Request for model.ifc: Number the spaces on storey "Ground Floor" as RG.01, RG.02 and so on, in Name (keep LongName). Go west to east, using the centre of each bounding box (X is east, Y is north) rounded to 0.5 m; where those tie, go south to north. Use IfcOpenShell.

First a look at what the model holds.

```python
import ifcopenshell
import ifcopenshell.util.element
import ifcopenshell.util.placement

model = ifcopenshell.open("model.ifc")
print(model.schema)
storey = next(s for s in model.by_type("IfcBuildingStorey") if s.Name == "Ground Floor")
spaces = [e for e in ifcopenshell.util.element.get_decomposition(storey) if e.is_a("IfcSpace")]
for e in sorted(spaces, key=lambda e: e.id()):
    origin = ifcopenshell.util.placement.get_local_placement(e.ObjectPlacement)[:3, 3]
    print(e.id(), e.Name, e.LongName, origin.round(2) + 0.0, sep=" | ")
```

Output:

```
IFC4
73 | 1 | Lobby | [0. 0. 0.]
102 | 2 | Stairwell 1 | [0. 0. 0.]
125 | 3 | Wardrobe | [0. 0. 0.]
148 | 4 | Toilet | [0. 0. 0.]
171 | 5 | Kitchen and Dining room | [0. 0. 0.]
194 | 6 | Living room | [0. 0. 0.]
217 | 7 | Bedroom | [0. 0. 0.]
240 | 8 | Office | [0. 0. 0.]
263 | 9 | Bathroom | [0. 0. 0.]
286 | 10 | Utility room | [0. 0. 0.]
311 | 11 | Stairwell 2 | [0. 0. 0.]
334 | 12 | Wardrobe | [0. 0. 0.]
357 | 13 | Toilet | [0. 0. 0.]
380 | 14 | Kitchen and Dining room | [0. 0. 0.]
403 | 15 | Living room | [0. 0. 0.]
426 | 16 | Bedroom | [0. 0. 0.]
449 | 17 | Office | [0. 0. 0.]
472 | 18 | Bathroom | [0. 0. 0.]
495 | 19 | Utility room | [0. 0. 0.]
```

```python
import ifcopenshell
import ifcopenshell.geom
import ifcopenshell.util.element
import ifcopenshell.util.shape

model = ifcopenshell.open("model.ifc")
settings = ifcopenshell.geom.settings()
settings.set("use-world-coords", True)


def centre(element):
    shape = ifcopenshell.geom.create_shape(settings, element)
    return ifcopenshell.util.shape.get_bbox_centroid(shape.geometry)


storey = next(s for s in model.by_type("IfcBuildingStorey") if s.Name == "Ground Floor")
spaces = [e for e in ifcopenshell.util.element.get_decomposition(storey) if e.is_a("IfcSpace")]

# Insertion points can sit at a corner or the storey origin, so sort by the geometry (in metres).
centres = {e: centre(e) for e in spaces}
spaces.sort(key=lambda e: (round(centres[e][0] / 0.5), centres[e][1]))

for i, e in enumerate(spaces, start=1):
    number = f"RG.{i:02d}"
    e.Name = number
    print(e.id(), number)

model.write("model_v2.ifc")
```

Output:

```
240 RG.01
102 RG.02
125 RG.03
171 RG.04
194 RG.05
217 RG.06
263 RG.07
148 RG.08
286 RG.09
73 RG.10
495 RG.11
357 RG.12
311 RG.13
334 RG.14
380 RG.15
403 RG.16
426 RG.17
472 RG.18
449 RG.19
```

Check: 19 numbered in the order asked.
